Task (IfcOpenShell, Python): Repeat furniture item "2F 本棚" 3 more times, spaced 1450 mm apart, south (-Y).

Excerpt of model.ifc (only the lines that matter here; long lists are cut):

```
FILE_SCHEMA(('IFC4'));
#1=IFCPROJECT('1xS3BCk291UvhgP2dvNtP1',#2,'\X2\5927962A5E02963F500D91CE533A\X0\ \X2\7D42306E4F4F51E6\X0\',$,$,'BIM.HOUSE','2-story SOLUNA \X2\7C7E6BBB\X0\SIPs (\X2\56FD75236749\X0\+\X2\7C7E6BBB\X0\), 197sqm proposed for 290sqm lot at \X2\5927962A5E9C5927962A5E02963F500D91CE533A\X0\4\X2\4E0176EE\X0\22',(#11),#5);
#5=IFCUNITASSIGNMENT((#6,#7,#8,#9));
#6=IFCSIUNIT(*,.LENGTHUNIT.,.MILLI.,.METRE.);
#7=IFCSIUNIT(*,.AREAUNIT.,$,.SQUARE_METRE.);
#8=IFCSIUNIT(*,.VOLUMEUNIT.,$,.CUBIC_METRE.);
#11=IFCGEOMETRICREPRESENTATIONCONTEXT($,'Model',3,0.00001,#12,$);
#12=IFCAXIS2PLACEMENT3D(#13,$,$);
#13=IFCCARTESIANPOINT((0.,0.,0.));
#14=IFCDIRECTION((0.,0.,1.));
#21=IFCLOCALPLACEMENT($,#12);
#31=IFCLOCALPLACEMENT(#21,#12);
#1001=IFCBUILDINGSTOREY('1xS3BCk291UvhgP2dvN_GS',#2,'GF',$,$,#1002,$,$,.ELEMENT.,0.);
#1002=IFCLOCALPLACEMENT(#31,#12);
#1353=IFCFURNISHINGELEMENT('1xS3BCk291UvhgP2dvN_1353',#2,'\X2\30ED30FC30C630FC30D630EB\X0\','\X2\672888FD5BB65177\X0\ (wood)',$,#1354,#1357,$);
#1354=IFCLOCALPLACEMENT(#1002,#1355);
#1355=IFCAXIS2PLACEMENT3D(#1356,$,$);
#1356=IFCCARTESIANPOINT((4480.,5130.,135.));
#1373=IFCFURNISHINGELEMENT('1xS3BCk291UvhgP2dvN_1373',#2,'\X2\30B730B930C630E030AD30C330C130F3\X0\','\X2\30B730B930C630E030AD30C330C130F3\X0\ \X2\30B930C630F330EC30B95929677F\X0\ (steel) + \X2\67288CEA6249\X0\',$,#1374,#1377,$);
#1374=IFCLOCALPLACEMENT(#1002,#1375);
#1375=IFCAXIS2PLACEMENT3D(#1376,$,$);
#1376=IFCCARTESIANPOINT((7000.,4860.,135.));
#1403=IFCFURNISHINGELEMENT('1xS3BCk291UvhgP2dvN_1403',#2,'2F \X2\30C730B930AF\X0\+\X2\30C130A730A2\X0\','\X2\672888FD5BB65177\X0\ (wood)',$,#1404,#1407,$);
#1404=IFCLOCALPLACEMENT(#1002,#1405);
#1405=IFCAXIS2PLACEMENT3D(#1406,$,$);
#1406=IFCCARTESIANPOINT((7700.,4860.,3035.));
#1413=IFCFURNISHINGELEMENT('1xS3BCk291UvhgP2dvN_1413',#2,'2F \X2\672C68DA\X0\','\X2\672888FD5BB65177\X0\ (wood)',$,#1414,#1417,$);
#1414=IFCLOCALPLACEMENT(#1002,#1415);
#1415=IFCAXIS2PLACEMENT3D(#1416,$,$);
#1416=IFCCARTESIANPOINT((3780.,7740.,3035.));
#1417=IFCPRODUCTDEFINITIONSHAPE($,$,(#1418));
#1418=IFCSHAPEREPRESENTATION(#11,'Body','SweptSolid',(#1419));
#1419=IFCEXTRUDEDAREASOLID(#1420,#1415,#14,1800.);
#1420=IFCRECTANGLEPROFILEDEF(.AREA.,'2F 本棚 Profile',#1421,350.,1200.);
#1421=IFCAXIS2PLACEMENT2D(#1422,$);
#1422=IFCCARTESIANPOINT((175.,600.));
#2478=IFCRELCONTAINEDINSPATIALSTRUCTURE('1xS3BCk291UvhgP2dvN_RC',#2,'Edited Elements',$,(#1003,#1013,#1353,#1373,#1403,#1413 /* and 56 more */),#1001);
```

```python
import numpy as np
import ifcopenshell
import ifcopenshell.api.geometry
import ifcopenshell.api.root
import ifcopenshell.util.element
import ifcopenshell.util.placement
import ifcopenshell.util.unit

model = ifcopenshell.open("model.ifc")
unit_scale = ifcopenshell.util.unit.calculate_unit_scale(model)


def reuse_history(source, copy):
    """copy_class also copies each property set's owner history, people and application; keep the originals."""
    for rel in copy.IsDefinedBy:
        if rel.is_a("IfcRelDefinesByProperties") and (history := rel.RelatingPropertyDefinition.OwnerHistory):
            rel.RelatingPropertyDefinition.OwnerHistory = source.OwnerHistory
            ifcopenshell.util.element.remove_deep2(model, history)


source = model.by_guid("1xS3BCk291UvhgP2dvN_1413")
base = ifcopenshell.util.placement.get_local_placement(source.ObjectPlacement)
step = np.array([0.0, -1.0, 0.0]) * 1.45 / unit_scale

for i in range(1, 4):
    copy = ifcopenshell.api.root.copy_class(model, product=source)
    copy.Representation = ifcopenshell.util.element.copy_deep(
        model, source.Representation, exclude=["IfcGeometricRepresentationContext", "IfcRepresentationMap"]
    )
    reuse_history(source, copy)
    matrix = base.copy()
    matrix[:3, 3] += i * step
    print("added at", matrix[:3, 3].round(3) + 0.0)
    ifcopenshell.api.geometry.edit_object_placement(model, product=copy, matrix=matrix, is_si=False)

model.write("model_updated.ifc")
```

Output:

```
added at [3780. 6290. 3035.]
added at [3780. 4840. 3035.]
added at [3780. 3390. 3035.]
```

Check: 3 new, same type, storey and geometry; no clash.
